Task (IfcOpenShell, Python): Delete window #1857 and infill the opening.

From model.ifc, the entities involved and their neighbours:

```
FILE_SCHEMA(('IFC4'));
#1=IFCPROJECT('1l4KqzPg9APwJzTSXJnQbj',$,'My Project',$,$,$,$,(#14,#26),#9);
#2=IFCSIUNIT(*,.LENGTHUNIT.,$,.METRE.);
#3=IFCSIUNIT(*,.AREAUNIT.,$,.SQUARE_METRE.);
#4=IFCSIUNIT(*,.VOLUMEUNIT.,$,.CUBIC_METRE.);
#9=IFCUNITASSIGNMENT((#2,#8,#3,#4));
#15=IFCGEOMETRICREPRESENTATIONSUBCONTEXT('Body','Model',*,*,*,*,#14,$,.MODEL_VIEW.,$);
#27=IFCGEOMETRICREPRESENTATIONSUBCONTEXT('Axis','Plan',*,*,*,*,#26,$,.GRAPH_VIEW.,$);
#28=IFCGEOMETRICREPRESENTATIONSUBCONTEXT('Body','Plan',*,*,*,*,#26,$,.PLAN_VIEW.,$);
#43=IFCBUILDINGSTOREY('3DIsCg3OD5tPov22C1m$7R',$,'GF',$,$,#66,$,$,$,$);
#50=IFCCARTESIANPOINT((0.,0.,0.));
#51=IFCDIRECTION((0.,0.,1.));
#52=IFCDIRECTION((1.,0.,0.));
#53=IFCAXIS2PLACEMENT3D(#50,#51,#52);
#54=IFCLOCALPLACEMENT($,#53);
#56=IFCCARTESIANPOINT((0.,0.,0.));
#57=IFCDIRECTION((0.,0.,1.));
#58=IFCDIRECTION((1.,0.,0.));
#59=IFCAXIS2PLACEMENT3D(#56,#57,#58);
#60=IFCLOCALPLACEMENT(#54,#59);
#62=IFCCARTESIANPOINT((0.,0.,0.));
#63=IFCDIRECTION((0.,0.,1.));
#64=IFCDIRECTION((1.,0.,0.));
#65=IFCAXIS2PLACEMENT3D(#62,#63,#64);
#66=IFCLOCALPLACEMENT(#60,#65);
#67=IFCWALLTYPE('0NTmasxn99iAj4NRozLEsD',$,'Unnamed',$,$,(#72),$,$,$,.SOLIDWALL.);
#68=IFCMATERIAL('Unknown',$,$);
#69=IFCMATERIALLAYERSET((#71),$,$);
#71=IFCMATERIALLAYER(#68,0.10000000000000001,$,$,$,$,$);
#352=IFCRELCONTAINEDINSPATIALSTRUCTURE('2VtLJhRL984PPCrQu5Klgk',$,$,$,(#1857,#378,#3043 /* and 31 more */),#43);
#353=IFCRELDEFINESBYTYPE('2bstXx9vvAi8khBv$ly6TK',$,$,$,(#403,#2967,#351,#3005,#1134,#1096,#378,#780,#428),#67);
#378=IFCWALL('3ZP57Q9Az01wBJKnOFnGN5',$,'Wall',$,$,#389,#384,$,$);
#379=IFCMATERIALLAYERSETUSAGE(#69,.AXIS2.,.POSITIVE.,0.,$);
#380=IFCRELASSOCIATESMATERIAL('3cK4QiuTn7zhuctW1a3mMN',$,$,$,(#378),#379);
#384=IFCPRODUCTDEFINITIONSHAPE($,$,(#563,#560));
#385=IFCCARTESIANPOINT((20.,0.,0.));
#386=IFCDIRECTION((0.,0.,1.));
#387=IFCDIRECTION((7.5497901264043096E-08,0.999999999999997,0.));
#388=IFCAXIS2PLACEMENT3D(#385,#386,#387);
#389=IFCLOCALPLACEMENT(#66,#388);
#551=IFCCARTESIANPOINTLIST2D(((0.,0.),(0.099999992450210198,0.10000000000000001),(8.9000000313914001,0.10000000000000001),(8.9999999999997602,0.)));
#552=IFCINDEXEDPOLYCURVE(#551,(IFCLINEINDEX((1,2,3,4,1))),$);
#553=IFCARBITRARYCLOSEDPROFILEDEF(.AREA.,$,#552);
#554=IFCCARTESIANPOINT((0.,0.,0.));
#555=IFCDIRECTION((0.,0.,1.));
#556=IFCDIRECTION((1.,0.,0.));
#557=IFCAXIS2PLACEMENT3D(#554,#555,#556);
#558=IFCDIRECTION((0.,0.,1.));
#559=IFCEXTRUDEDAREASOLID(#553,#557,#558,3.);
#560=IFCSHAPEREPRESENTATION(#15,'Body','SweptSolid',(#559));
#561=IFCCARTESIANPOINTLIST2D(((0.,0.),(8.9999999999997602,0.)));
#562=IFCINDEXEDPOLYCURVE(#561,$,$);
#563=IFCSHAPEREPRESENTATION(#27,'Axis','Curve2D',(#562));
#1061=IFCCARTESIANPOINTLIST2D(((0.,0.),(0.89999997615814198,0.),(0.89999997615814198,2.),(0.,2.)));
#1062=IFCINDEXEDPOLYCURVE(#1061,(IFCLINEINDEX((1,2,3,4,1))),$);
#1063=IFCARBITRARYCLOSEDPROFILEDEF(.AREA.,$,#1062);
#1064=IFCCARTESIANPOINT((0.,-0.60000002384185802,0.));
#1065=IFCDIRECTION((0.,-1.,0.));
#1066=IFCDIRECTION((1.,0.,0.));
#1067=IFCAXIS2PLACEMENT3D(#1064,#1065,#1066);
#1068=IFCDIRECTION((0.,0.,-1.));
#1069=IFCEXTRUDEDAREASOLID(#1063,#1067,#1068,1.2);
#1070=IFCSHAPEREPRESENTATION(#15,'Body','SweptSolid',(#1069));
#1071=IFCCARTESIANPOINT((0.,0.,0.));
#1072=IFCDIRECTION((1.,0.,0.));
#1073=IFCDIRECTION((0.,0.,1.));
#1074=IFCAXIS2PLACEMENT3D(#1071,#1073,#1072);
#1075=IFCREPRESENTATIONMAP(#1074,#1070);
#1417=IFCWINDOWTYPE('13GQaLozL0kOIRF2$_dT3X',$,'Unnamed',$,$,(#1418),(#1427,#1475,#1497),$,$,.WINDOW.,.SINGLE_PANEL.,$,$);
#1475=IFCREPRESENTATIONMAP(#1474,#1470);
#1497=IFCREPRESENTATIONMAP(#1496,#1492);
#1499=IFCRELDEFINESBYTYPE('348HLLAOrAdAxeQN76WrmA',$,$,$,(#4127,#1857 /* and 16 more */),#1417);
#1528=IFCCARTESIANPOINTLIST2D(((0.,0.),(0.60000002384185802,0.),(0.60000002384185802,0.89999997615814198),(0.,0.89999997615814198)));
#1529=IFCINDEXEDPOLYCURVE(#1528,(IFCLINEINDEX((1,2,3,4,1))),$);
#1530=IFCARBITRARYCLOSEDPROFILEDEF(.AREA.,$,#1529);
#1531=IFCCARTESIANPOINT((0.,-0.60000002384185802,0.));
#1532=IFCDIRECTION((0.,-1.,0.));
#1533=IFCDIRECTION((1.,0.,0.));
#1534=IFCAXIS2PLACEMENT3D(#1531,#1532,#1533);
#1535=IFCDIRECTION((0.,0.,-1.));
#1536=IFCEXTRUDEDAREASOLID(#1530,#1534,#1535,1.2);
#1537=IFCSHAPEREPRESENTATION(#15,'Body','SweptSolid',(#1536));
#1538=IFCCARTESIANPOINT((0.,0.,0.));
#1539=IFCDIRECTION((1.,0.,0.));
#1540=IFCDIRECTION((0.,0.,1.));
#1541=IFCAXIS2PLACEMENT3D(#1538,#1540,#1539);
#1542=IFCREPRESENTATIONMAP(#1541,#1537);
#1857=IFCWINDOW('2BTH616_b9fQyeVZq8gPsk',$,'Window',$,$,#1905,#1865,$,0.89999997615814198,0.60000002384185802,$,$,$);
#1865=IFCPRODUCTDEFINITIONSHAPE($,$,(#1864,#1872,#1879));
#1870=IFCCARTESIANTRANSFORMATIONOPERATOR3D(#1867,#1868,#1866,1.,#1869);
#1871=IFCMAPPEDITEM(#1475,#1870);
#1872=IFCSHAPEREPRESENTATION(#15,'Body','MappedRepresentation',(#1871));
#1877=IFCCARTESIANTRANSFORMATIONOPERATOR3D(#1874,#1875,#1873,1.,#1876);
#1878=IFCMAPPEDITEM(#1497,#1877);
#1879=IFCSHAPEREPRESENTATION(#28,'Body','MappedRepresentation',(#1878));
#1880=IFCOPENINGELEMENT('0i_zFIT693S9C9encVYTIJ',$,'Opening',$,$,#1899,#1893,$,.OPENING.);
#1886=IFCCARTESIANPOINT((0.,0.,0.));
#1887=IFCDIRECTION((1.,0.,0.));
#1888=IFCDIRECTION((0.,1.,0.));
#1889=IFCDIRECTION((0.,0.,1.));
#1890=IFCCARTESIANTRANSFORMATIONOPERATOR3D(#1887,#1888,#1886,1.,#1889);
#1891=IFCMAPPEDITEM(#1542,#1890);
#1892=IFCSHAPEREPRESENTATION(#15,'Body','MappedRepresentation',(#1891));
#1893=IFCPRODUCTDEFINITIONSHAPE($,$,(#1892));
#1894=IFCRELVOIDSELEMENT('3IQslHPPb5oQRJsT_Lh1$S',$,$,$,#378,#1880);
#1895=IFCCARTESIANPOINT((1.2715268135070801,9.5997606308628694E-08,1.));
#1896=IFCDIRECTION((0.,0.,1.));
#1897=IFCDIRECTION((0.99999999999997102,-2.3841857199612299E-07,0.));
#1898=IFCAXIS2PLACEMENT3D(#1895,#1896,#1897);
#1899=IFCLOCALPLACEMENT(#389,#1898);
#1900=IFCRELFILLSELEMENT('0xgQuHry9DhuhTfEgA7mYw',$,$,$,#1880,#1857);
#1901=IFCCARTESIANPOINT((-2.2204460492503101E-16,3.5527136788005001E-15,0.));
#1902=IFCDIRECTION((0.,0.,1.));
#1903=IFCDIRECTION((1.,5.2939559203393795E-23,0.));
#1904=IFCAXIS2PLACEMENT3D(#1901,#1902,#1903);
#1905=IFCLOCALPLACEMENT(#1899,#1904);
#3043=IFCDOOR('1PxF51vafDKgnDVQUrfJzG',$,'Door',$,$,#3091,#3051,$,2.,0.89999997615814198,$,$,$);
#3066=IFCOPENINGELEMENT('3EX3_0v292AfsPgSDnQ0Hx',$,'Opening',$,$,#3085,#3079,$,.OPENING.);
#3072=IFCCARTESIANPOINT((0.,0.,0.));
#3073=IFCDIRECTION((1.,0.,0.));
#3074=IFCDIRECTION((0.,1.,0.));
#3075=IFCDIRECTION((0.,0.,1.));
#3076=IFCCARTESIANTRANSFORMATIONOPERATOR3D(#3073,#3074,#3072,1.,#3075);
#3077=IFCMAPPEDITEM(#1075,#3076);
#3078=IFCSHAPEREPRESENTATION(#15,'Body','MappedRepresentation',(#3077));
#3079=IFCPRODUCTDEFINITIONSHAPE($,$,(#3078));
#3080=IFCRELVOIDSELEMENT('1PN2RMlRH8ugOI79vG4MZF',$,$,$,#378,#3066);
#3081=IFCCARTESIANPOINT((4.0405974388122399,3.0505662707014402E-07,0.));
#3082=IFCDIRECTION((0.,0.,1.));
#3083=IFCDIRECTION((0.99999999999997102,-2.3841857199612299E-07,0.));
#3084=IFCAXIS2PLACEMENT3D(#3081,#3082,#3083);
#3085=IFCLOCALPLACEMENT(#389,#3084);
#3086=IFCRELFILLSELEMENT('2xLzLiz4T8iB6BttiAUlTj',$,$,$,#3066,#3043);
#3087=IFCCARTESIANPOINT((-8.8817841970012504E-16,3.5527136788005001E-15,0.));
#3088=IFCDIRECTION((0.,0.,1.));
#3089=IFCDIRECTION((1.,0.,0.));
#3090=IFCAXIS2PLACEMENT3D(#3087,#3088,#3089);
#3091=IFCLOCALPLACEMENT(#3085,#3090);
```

```python
import ifcopenshell
import ifcopenshell.api.feature
import ifcopenshell.api.root
import ifcopenshell.geom
import ifcopenshell.util.shape

model = ifcopenshell.open("model.ifc")
settings = ifcopenshell.geom.settings()


def volume(element):
    """Net volume in cubic metres, openings subtracted."""
    shape = ifcopenshell.geom.create_shape(settings, element)
    return ifcopenshell.util.shape.get_volume(shape.geometry)


window = model.by_guid("2BTH616_b9fQyeVZq8gPsk")
opening = window.FillsVoids[0].RelatingOpeningElement
wall = opening.VoidsElements[0].RelatingBuildingElement
before = volume(wall)

ifcopenshell.api.root.remove_product(model, product=window)
ifcopenshell.api.feature.remove_feature(model, feature=opening)

after = volume(wall)

print(f"wall volume {before:.3f} -> {after:.3f} m3")

model.write("model_updated.ifc")
```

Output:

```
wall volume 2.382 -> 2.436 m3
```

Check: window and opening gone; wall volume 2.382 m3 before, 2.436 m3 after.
